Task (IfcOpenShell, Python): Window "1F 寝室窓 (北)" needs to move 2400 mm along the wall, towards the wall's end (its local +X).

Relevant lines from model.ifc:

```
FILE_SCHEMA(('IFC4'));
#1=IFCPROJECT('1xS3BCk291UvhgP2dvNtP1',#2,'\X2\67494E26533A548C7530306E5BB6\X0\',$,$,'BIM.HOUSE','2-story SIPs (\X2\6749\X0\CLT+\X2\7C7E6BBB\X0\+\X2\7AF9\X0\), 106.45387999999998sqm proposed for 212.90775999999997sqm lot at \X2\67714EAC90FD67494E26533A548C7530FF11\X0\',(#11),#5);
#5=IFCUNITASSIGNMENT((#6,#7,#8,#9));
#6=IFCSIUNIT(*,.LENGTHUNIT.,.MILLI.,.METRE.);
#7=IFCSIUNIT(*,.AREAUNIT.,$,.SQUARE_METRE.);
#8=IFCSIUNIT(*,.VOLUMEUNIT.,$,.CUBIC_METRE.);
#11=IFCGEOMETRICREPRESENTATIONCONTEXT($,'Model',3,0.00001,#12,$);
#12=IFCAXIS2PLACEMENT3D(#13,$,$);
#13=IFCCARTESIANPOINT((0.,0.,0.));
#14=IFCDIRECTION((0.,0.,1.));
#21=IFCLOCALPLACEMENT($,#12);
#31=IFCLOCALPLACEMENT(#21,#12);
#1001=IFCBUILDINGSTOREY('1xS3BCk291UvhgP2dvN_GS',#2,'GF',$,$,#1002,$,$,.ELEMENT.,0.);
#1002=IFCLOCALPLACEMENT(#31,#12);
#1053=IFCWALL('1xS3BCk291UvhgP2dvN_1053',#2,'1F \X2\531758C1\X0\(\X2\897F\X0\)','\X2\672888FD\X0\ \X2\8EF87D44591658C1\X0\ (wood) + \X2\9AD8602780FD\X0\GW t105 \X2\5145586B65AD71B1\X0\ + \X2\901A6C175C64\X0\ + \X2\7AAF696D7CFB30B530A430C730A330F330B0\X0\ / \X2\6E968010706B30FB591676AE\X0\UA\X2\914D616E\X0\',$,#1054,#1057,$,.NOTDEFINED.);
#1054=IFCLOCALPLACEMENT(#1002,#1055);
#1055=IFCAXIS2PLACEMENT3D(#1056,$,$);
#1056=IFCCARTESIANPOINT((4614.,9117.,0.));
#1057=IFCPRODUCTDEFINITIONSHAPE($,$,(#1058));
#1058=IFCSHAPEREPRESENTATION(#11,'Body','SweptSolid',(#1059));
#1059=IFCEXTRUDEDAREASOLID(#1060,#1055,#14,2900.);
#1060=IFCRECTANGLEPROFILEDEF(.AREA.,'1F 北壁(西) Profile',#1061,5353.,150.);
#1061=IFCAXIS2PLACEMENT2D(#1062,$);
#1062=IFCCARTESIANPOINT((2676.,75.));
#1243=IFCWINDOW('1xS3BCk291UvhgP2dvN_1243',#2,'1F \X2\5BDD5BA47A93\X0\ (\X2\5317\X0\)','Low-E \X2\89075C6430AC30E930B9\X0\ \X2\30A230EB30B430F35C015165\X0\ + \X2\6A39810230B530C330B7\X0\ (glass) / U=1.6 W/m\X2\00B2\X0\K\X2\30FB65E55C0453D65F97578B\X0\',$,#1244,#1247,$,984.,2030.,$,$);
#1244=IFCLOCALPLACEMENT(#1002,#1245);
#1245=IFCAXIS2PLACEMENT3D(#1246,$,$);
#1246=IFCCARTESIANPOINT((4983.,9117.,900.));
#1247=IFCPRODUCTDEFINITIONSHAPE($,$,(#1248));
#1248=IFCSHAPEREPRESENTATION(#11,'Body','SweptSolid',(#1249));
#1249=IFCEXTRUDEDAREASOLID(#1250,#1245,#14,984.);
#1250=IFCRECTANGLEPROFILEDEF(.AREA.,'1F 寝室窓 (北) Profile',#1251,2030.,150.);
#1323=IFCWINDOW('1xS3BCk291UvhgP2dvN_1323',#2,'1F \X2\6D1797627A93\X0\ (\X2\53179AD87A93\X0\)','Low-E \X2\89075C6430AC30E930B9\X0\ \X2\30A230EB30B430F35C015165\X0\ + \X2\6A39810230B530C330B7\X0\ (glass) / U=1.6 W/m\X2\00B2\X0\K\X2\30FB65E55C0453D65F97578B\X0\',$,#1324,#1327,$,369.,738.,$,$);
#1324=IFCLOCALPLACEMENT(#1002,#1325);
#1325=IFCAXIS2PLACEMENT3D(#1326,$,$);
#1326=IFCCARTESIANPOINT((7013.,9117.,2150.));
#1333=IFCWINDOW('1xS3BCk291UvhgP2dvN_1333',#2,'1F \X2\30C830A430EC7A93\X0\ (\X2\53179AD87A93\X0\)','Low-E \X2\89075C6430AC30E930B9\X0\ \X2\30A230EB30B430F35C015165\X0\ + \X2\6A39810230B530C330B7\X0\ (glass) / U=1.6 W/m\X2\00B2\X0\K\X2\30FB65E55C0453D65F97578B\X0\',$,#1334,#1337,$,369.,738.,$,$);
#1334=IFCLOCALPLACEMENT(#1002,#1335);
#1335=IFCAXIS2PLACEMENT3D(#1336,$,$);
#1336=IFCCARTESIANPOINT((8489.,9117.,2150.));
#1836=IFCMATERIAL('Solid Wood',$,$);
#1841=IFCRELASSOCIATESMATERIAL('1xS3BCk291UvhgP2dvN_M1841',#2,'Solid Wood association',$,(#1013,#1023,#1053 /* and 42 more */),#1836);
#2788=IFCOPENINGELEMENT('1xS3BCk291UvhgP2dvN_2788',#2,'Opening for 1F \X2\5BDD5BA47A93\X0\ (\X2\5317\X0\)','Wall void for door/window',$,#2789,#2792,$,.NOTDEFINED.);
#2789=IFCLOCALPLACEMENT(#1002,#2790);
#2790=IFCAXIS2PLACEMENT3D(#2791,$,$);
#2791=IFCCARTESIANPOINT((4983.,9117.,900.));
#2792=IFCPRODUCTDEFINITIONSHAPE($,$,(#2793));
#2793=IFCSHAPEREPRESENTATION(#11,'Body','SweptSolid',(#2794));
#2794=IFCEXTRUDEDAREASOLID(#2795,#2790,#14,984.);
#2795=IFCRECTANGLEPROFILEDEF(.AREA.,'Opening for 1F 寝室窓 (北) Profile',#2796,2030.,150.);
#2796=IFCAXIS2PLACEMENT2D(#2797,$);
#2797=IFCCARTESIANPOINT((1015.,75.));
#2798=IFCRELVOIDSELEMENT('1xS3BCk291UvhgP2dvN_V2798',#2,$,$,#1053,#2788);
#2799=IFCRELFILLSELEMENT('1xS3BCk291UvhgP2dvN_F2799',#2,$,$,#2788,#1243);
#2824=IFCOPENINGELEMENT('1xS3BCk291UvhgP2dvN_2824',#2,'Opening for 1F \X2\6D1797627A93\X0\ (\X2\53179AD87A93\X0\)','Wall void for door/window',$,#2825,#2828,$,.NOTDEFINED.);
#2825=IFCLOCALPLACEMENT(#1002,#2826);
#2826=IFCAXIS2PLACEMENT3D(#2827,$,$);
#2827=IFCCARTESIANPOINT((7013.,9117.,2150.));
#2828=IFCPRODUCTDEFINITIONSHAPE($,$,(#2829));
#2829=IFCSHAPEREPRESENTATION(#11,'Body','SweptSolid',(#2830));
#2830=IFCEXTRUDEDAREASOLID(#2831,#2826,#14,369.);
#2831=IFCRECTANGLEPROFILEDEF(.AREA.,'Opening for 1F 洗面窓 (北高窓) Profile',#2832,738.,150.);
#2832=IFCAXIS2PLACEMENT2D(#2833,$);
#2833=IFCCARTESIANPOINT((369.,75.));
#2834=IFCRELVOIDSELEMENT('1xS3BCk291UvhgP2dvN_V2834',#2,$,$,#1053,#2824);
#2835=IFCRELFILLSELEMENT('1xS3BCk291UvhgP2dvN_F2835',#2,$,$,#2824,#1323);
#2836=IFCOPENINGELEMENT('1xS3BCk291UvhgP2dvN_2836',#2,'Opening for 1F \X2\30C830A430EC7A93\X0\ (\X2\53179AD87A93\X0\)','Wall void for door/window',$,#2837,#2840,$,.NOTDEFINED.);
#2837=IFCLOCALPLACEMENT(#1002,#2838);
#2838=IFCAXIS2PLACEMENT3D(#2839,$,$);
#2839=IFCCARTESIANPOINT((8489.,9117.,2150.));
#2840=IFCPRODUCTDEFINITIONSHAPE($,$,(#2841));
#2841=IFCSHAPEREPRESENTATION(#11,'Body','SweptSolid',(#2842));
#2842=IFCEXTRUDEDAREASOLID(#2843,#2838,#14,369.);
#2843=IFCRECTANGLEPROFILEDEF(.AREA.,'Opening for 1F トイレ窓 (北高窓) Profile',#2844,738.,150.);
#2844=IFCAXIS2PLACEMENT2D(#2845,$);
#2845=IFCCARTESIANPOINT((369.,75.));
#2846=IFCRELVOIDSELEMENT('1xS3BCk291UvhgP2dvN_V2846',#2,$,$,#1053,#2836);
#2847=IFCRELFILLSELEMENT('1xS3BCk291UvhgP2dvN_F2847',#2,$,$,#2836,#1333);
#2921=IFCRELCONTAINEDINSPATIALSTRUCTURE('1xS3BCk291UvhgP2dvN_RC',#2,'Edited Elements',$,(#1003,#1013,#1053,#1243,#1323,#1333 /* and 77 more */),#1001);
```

```python
import ifcopenshell
import ifcopenshell.api.geometry
import ifcopenshell.util.placement

model = ifcopenshell.open("model.ifc")

window = model.by_guid("1xS3BCk291UvhgP2dvN_1243")
opening = window.FillsVoids[0].RelatingOpeningElement
wall = opening.VoidsElements[0].RelatingBuildingElement

wall_matrix = ifcopenshell.util.placement.get_local_placement(wall.ObjectPlacement)
shift = wall_matrix[:3, 0] * 2400.0
before = ifcopenshell.util.placement.get_local_placement(window.ObjectPlacement)[:3, 3].copy()

# The window is not placed relative to its opening, so move both.
for product in (opening, window):
    matrix = ifcopenshell.util.placement.get_local_placement(product.ObjectPlacement)
    matrix[:3, 3] += shift
    ifcopenshell.api.geometry.edit_object_placement(model, product=product, matrix=matrix, is_si=False)

after = ifcopenshell.util.placement.get_local_placement(window.ObjectPlacement)[:3, 3]
print("window moved by", (after - before).round(3) + 0.0)

model.write("model-out.ifc")
```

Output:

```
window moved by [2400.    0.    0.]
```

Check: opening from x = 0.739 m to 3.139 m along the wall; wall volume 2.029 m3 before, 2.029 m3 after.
